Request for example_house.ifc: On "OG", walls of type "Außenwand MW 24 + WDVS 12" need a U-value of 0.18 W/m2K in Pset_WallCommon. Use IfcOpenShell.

First a look at what the model holds.

```python
import ifcopenshell
import ifcopenshell.util.element

model = ifcopenshell.open("example_house.ifc")
print(model.schema)
storey = next(s for s in model.by_type("IfcBuildingStorey") if s.Name == "OG")
walls = [e for e in ifcopenshell.util.element.get_decomposition(storey) if e.is_a("IfcWall")]
seen = {}
for e in walls:
    element_type = ifcopenshell.util.element.get_type(e)
    key = (element_type.Name if element_type != e and element_type else None, ifcopenshell.util.element.get_pset(e, "Pset_WallCommon", "ThermalTransmittance"))
    seen[key] = seen.get(key, 0) + 1
for (name, value), count in sorted(seen.items(), key=str):
    print(count, "x", name, "|", value)
```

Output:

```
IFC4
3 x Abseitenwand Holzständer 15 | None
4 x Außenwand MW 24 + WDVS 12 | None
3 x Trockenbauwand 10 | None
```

```python
import ifcopenshell
import ifcopenshell.api.pset
import ifcopenshell.util.element

model = ifcopenshell.open("example_house.ifc")

storey = next(s for s in model.by_type("IfcBuildingStorey") if s.Name == "OG")
walls = [e for e in ifcopenshell.util.element.get_decomposition(storey) if e.is_a("IfcWall")]

count = 0
for e in walls:
    element_type = ifcopenshell.util.element.get_type(e)
    if element_type in (None, e) or element_type.Name != "Außenwand MW 24 + WDVS 12":
        continue
    # add_pset returns the element's existing set when there is one.
    pset = ifcopenshell.api.pset.add_pset(model, product=e, name="Pset_WallCommon")
    ifcopenshell.api.pset.edit_pset(model, pset=pset, properties={"ThermalTransmittance": 0.18})
    count += 1

print(count, "walls updated")

model.write("example_house_rev.ifc")
```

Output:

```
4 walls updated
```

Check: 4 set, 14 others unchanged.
